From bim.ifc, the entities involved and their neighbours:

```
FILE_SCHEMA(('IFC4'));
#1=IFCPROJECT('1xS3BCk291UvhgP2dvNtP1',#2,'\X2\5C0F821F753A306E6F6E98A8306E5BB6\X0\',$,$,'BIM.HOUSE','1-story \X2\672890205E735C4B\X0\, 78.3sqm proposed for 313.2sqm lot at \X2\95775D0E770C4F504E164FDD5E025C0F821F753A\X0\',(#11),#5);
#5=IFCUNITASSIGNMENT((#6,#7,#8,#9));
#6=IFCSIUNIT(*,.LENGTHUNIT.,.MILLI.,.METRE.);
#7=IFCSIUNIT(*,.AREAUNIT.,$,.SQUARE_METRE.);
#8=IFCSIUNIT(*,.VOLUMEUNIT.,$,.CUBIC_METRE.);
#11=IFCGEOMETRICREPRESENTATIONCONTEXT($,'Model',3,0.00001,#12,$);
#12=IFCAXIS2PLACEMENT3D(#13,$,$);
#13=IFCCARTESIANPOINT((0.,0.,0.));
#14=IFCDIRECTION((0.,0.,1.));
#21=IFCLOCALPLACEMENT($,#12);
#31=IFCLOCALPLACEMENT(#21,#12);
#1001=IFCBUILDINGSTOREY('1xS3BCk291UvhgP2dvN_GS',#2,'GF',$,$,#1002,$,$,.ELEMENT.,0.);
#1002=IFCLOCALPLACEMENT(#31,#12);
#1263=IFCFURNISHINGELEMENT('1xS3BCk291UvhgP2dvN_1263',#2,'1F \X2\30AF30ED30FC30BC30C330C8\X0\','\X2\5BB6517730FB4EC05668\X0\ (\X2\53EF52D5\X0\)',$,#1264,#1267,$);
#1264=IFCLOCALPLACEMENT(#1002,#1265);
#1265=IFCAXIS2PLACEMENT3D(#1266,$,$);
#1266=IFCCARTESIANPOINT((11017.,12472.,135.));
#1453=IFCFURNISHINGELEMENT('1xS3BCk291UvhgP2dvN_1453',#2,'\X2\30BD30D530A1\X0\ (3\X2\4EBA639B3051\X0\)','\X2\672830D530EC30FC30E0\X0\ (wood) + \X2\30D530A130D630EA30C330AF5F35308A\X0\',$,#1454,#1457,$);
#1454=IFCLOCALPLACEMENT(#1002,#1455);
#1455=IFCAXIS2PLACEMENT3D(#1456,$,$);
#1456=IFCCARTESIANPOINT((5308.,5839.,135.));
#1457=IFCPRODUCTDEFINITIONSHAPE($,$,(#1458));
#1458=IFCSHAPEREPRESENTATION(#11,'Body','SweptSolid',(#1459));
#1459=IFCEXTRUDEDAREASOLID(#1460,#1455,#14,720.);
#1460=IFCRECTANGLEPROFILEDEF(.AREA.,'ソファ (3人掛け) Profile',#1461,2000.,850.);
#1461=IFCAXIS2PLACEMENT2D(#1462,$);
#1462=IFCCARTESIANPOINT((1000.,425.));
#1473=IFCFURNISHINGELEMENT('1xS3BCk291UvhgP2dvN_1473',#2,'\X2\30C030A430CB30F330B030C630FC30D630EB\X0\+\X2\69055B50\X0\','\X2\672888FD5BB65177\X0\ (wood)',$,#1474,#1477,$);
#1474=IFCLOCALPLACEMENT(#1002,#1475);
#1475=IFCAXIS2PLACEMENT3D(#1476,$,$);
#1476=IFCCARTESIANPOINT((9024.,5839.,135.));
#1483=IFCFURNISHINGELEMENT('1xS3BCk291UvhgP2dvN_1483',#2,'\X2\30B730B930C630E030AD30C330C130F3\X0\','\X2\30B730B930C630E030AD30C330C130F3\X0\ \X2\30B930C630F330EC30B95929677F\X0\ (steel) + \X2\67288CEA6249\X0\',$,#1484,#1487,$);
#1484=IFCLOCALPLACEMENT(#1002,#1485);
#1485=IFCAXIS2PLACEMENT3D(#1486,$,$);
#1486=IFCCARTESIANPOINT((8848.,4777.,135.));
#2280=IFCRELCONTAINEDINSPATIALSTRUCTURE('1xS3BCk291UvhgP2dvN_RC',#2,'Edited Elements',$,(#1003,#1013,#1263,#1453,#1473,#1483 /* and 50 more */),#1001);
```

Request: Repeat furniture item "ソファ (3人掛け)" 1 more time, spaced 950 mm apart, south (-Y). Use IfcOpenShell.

```python
import numpy as np
import ifcopenshell
import ifcopenshell.api.geometry
import ifcopenshell.api.root
import ifcopenshell.util.element
import ifcopenshell.util.placement

model = ifcopenshell.open("bim.ifc")


def reuse_history(source, copy):
    """copy_class also copies each property set's owner history, people and application; keep the originals."""
    for rel in copy.IsDefinedBy:
        if rel.is_a("IfcRelDefinesByProperties") and (history := rel.RelatingPropertyDefinition.OwnerHistory):
            rel.RelatingPropertyDefinition.OwnerHistory = source.OwnerHistory
            ifcopenshell.util.element.remove_deep2(model, history)


source = model.by_id(1453)
base = ifcopenshell.util.placement.get_local_placement(source.ObjectPlacement)
step = np.array([0.0, -1.0, 0.0]) * 950.0

for i in range(1, 2):
    copy = ifcopenshell.api.root.copy_class(model, product=source)
    copy.Representation = ifcopenshell.util.element.copy_deep(
        model, source.Representation, exclude=["IfcGeometricRepresentationContext", "IfcRepresentationMap"]
    )
    reuse_history(source, copy)
    matrix = base.copy()
    matrix[:3, 3] += i * step
    print("added at", matrix[:3, 3].round(3) + 0.0)
    ifcopenshell.api.geometry.edit_object_placement(model, product=copy, matrix=matrix, is_si=False)

model.write("bim_rev.ifc")
```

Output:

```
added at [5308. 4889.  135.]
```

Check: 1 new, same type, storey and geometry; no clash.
